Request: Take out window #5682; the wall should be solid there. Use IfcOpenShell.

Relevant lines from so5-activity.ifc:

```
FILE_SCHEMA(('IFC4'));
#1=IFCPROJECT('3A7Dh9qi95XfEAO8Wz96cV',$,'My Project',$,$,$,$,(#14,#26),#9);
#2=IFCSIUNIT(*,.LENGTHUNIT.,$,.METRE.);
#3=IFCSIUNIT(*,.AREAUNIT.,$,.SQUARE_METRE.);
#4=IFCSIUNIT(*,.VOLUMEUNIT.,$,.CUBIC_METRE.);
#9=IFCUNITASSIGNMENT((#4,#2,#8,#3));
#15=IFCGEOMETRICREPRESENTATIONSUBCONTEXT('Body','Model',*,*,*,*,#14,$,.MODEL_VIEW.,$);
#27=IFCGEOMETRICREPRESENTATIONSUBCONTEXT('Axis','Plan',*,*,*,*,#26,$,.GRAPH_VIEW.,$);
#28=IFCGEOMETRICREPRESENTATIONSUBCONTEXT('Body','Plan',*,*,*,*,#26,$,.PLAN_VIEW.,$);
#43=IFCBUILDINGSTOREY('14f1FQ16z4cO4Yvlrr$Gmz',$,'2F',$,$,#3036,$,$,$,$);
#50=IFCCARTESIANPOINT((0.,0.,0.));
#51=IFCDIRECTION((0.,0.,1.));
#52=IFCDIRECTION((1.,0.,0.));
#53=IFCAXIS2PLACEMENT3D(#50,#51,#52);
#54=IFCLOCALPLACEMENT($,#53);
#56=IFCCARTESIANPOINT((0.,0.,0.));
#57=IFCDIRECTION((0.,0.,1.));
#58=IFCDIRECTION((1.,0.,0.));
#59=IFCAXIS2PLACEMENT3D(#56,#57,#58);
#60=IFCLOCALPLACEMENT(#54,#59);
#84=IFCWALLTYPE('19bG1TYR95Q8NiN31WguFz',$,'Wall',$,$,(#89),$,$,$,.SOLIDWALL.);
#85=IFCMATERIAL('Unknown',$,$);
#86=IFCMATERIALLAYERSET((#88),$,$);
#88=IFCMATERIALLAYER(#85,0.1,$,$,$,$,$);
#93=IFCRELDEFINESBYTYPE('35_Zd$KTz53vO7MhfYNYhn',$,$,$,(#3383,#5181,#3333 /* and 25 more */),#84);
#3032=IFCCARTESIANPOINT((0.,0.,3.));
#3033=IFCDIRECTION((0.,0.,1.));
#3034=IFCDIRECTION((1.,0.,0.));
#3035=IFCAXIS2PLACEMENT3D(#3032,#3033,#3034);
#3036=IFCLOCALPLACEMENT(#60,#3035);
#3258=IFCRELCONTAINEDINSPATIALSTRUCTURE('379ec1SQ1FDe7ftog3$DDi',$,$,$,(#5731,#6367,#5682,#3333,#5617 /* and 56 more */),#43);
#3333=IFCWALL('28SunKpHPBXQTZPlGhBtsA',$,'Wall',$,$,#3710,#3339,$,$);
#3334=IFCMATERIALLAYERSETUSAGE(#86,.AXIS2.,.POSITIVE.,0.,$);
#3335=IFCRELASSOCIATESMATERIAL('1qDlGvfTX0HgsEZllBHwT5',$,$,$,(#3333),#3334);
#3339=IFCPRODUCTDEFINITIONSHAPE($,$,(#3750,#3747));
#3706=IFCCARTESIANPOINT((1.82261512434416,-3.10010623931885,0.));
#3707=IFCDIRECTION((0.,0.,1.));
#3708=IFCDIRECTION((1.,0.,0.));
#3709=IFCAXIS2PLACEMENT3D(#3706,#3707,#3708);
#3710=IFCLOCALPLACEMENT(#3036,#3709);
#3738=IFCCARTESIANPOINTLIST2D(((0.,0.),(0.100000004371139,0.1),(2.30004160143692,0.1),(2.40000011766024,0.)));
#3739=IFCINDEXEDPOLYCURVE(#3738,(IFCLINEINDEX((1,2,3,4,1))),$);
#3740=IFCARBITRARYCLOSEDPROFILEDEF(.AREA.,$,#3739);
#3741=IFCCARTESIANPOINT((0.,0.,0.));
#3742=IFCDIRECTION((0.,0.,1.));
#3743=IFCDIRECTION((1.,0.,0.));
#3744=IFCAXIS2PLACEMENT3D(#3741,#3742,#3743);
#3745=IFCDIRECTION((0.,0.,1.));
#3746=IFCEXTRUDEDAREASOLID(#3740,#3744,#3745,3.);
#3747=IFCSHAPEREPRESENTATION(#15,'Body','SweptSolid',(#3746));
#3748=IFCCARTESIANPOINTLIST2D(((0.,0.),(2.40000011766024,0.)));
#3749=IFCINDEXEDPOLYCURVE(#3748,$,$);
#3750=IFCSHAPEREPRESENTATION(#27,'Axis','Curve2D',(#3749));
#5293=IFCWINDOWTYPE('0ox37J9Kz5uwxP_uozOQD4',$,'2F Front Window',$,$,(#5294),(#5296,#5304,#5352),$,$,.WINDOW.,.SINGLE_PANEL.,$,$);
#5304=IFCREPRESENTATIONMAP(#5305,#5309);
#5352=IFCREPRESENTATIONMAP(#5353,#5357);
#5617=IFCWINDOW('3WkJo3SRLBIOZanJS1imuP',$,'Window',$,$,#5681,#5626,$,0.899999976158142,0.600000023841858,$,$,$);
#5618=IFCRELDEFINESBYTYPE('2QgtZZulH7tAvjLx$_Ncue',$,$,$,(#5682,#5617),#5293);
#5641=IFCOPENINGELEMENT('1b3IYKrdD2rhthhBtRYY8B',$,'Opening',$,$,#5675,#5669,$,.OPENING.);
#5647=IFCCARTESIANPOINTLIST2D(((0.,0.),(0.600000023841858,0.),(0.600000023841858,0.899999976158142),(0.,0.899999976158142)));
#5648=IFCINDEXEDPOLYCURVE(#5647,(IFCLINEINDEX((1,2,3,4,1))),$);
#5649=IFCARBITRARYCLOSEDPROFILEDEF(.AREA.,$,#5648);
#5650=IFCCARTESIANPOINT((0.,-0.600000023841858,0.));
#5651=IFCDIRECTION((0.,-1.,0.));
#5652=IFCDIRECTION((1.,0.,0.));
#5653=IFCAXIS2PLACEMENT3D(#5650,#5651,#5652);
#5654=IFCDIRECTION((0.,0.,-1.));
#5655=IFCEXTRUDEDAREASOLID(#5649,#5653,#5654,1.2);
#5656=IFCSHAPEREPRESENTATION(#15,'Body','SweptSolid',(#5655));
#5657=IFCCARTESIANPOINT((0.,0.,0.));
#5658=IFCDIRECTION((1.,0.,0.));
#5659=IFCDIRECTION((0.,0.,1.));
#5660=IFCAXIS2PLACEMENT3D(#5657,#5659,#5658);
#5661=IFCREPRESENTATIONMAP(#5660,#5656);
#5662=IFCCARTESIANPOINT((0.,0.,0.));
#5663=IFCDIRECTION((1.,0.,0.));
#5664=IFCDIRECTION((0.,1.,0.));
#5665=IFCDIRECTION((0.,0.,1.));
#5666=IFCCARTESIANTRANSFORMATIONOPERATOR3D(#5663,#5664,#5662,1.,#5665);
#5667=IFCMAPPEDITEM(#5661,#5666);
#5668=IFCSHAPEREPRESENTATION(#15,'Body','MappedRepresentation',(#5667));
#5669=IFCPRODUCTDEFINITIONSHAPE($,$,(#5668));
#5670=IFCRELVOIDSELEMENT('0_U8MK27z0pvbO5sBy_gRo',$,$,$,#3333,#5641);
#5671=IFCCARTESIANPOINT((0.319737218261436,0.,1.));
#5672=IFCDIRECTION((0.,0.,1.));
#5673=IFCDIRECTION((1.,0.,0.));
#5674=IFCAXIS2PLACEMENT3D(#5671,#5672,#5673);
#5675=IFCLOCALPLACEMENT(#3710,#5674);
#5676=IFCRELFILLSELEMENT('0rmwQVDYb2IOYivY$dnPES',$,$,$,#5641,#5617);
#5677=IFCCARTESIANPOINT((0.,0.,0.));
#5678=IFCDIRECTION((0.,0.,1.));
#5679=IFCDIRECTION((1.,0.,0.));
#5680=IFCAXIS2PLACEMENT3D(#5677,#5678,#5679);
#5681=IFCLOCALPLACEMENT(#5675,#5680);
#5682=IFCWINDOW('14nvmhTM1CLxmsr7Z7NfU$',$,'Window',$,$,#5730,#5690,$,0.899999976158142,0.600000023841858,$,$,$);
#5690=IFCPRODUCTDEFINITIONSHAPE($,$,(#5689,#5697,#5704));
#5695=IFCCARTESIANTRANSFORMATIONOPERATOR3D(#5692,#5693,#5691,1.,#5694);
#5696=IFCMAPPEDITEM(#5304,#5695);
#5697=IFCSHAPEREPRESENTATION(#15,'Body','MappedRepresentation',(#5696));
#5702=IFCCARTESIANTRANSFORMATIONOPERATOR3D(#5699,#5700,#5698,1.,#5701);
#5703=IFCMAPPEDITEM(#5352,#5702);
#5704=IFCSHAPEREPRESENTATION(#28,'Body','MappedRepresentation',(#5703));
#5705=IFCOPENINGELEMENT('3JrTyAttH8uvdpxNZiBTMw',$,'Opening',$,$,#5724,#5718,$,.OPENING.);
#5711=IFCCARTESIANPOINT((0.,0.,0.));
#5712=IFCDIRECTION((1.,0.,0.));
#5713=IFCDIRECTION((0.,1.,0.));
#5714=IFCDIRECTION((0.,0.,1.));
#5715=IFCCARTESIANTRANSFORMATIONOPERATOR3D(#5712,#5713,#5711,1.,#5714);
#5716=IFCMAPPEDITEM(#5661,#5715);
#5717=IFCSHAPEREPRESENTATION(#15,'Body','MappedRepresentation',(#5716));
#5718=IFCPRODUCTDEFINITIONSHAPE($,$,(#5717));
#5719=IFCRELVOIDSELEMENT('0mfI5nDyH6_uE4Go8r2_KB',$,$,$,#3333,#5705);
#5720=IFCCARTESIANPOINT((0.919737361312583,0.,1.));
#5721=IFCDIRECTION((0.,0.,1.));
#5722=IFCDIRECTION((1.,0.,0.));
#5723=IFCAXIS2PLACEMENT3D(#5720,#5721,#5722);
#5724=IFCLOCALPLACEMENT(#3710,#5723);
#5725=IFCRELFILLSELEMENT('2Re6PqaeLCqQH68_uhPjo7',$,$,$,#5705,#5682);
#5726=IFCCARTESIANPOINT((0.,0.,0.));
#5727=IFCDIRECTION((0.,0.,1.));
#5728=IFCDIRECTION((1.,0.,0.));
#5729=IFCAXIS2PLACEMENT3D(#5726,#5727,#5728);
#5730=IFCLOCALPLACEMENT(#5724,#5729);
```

```python
import ifcopenshell
import ifcopenshell.api.feature
import ifcopenshell.api.root
import ifcopenshell.geom
import ifcopenshell.util.shape

model = ifcopenshell.open("so5-activity.ifc")
settings = ifcopenshell.geom.settings()


def volume(element):
    """Net volume in cubic metres, openings subtracted."""
    shape = ifcopenshell.geom.create_shape(settings, element)
    return ifcopenshell.util.shape.get_volume(shape.geometry)


window = model.by_guid("14nvmhTM1CLxmsr7Z7NfU$")
opening = window.FillsVoids[0].RelatingOpeningElement
wall = opening.VoidsElements[0].RelatingBuildingElement
before = volume(wall)

ifcopenshell.api.root.remove_product(model, product=window)
ifcopenshell.api.feature.remove_feature(model, feature=opening)

after = volume(wall)

print(f"wall volume {before:.3f} -> {after:.3f} m3")

model.write("so5-activity_v2.ifc")
```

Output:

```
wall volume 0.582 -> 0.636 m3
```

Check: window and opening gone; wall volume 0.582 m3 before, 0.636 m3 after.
